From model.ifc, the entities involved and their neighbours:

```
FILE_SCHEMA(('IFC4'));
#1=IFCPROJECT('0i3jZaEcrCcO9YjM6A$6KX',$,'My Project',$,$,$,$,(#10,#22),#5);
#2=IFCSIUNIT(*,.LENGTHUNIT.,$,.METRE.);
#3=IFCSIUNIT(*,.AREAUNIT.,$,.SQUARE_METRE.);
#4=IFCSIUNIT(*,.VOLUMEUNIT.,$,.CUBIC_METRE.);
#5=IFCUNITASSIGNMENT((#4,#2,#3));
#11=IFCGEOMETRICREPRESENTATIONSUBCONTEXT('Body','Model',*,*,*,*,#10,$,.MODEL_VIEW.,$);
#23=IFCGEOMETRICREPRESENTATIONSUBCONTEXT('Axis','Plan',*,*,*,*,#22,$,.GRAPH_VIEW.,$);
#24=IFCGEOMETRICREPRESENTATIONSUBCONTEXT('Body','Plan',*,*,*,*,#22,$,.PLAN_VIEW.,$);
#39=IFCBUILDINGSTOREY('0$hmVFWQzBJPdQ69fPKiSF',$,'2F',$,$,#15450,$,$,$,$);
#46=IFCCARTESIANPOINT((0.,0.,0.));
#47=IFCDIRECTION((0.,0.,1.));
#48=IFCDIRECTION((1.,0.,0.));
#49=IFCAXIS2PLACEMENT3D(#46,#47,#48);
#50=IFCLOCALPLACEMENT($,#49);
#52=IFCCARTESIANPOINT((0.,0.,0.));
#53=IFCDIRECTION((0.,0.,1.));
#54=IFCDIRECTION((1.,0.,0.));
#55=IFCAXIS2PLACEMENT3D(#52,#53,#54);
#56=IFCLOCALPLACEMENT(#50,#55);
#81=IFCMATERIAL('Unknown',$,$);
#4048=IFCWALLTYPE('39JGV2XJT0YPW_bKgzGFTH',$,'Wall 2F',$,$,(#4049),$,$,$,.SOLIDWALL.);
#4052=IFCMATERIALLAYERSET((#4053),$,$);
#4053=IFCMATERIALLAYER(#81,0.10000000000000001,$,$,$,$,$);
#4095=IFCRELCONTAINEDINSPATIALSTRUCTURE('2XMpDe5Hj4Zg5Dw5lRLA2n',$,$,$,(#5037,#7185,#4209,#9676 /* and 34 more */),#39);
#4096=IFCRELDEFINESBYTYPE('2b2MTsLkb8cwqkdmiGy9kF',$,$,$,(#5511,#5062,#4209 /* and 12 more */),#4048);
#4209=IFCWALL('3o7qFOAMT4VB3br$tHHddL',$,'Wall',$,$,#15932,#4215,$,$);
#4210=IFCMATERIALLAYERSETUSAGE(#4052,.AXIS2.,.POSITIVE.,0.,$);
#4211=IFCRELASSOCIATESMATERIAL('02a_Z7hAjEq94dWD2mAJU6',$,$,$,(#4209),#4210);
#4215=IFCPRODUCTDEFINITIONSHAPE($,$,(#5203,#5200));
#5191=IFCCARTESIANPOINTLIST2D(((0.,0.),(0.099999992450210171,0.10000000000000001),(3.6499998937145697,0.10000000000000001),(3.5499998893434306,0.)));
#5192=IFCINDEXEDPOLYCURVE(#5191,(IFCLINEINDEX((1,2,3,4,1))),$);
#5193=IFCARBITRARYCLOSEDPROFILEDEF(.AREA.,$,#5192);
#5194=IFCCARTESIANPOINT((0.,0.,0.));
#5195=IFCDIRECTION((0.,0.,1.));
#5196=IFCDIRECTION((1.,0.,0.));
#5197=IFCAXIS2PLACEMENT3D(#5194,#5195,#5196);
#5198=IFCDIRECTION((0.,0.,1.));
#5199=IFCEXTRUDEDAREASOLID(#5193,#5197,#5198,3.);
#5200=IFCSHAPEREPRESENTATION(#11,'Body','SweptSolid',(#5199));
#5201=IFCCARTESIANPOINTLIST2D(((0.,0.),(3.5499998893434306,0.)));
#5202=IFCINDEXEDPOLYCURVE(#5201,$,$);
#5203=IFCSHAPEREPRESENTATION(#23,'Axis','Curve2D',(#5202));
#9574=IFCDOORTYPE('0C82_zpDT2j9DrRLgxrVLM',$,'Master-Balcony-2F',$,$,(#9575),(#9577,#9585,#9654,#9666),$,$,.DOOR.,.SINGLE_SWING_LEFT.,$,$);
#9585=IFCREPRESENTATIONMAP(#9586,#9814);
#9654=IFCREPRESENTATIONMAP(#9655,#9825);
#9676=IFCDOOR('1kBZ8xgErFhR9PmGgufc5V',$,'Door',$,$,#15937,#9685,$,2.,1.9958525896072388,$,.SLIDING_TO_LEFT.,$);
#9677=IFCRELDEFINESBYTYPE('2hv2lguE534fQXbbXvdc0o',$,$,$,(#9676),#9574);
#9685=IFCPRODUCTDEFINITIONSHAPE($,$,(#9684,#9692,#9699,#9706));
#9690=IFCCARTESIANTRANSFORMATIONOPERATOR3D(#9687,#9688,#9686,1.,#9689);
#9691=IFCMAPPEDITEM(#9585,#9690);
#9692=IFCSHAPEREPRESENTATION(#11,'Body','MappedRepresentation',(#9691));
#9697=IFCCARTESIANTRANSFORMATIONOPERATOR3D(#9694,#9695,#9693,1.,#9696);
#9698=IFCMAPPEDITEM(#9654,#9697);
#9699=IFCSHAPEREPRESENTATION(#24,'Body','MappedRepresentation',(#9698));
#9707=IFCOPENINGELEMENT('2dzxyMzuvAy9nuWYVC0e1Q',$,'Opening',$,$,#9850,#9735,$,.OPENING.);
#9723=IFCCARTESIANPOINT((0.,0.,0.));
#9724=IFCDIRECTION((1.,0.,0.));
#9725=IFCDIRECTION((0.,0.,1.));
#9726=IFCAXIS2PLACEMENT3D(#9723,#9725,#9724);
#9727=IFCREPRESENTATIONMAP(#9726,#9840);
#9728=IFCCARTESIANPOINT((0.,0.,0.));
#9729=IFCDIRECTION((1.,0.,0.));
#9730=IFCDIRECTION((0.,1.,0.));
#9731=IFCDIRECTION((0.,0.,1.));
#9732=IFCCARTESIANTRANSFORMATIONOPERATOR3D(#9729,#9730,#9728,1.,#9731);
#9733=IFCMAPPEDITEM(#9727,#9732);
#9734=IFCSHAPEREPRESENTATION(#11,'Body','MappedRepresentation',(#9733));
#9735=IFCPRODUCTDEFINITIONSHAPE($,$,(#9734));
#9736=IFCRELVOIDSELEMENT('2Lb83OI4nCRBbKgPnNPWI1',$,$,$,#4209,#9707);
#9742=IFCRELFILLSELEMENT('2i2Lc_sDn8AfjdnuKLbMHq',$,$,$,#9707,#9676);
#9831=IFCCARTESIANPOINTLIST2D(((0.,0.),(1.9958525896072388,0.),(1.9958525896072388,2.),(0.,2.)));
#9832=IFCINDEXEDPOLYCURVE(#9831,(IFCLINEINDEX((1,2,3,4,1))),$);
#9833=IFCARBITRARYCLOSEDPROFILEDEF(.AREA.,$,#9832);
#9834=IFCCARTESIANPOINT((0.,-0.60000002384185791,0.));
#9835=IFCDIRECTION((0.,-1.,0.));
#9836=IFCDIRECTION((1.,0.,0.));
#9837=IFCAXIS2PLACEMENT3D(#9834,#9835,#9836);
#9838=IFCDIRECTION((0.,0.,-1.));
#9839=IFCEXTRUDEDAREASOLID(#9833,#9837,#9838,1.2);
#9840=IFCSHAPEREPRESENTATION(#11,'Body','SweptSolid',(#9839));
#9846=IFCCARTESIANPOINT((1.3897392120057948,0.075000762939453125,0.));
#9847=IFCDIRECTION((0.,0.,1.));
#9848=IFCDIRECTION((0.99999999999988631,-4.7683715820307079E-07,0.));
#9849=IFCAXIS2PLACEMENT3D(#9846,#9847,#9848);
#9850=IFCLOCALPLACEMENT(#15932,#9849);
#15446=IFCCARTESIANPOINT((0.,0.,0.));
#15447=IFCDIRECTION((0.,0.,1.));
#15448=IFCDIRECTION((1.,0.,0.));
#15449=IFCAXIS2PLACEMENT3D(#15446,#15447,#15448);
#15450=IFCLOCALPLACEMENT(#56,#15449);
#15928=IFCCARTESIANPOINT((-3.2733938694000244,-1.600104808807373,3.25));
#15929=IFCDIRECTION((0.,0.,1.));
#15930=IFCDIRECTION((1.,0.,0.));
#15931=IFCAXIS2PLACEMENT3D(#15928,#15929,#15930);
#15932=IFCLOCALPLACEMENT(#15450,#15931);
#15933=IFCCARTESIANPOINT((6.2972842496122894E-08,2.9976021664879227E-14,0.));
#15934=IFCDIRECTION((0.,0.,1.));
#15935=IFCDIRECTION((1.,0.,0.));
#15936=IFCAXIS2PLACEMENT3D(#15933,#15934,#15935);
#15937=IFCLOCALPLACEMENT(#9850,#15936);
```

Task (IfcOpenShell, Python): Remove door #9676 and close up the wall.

```python
import ifcopenshell
import ifcopenshell.api.feature
import ifcopenshell.api.root
import ifcopenshell.geom
import ifcopenshell.util.shape

model = ifcopenshell.open("model.ifc")
settings = ifcopenshell.geom.settings()


def volume(element):
    """Net volume in cubic metres, openings subtracted."""
    shape = ifcopenshell.geom.create_shape(settings, element)
    return ifcopenshell.util.shape.get_volume(shape.geometry)


door = model.by_guid("1kBZ8xgErFhR9PmGgufc5V")
opening = door.FillsVoids[0].RelatingOpeningElement
wall = opening.VoidsElements[0].RelatingBuildingElement
before = volume(wall)

ifcopenshell.api.root.remove_product(model, product=door)
ifcopenshell.api.feature.remove_feature(model, feature=opening)

after = volume(wall)

print(f"wall volume {before:.3f} -> {after:.3f} m3")

model.write("model_rev.ifc")
```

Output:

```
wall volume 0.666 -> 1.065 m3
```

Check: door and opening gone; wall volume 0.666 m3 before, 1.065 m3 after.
